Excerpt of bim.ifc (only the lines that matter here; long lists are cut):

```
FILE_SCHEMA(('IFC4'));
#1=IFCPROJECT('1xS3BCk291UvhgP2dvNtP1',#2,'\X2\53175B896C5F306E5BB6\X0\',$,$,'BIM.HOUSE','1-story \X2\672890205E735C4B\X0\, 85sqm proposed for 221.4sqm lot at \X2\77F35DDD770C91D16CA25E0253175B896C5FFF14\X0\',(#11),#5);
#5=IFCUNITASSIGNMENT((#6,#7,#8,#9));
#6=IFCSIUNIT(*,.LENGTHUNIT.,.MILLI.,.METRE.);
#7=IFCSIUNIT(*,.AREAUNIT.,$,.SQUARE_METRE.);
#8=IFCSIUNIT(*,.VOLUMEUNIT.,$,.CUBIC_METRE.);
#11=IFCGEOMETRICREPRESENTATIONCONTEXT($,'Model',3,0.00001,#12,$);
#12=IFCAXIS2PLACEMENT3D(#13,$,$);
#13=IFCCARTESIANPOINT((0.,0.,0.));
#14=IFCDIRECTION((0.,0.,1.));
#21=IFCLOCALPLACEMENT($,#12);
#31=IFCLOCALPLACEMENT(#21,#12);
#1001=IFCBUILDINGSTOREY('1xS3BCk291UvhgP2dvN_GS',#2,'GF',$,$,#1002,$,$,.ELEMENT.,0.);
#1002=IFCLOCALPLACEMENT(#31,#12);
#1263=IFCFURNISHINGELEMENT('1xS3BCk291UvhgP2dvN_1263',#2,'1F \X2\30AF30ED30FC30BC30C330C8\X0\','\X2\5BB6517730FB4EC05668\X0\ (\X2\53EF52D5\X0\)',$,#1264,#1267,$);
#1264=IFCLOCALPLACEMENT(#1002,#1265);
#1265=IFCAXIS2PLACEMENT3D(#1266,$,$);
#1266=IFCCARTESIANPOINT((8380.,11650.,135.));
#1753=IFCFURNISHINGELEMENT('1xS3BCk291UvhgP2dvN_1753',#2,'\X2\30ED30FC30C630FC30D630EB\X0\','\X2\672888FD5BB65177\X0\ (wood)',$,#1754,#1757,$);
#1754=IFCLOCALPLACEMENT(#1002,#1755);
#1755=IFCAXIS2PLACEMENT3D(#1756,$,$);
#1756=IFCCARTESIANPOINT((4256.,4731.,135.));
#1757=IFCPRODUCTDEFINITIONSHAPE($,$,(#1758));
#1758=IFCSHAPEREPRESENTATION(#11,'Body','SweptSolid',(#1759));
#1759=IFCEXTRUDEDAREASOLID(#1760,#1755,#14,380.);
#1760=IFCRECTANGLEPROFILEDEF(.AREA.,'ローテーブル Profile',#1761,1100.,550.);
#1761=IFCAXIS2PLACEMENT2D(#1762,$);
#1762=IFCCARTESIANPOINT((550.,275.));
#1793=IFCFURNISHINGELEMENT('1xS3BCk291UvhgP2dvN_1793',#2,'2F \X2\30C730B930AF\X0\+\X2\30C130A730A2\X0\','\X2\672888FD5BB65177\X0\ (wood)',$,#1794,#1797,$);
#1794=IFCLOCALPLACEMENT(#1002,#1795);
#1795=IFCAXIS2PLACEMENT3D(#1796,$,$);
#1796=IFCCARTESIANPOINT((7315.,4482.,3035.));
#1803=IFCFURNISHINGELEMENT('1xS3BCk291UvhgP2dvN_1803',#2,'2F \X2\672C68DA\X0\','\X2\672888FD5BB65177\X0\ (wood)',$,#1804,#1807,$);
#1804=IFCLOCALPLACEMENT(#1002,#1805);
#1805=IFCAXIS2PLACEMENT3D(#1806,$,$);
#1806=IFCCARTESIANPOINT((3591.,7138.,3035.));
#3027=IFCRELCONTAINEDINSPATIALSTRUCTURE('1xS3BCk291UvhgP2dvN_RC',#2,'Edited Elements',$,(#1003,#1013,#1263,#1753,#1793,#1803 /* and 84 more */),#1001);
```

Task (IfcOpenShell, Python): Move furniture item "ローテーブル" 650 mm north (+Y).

```python
import ifcopenshell
import ifcopenshell.api.geometry
import ifcopenshell.util.placement

model = ifcopenshell.open("bim.ifc")

item = model.by_guid("1xS3BCk291UvhgP2dvN_1753")
matrix = ifcopenshell.util.placement.get_local_placement(item.ObjectPlacement)
matrix[1, 3] += 650.0
ifcopenshell.api.geometry.edit_object_placement(model, product=item, matrix=matrix, is_si=False)

print(ifcopenshell.util.placement.get_local_placement(item.ObjectPlacement).round(3) + 0.0)

model.write("bim-out.ifc")
```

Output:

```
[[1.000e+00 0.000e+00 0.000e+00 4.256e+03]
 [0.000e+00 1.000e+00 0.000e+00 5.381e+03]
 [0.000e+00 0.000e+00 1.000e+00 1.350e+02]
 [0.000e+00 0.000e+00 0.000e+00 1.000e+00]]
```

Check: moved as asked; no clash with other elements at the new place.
